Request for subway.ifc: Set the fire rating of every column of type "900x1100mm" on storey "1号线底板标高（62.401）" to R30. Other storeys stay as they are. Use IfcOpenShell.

First a look at what the model holds.

```python
import ifcopenshell
import ifcopenshell.util.element

model = ifcopenshell.open("subway.ifc")
print(model.schema)
storey = next(s for s in model.by_type("IfcBuildingStorey") if s.Name == "1号线底板标高（62.401）")
columns = [e for e in ifcopenshell.util.element.get_decomposition(storey) if e.is_a("IfcColumn")]
seen = {}
for e in columns:
    element_type = ifcopenshell.util.element.get_type(e)
    key = (element_type.Name if element_type != e and element_type else None, ifcopenshell.util.element.get_pset(e, "Pset_ColumnCommon", "FireRating"))
    seen[key] = seen.get(key, 0) + 1
for (name, value), count in sorted(seen.items(), key=str):
    print(count, "x", name, "|", value)
```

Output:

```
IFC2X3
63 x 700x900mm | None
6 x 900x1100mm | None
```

```python
import ifcopenshell
import ifcopenshell.api.pset
import ifcopenshell.util.element

model = ifcopenshell.open("subway.ifc")

storey = next(s for s in model.by_type("IfcBuildingStorey") if s.Name == "1号线底板标高（62.401）")
columns = [e for e in ifcopenshell.util.element.get_decomposition(storey) if e.is_a("IfcColumn")]

count = 0
for e in columns:
    element_type = ifcopenshell.util.element.get_type(e)
    if element_type in (None, e) or element_type.Name != "900x1100mm":
        continue
    # add_pset returns the element's existing set when there is one.
    pset = ifcopenshell.api.pset.add_pset(model, product=e, name="Pset_ColumnCommon")
    ifcopenshell.api.pset.edit_pset(model, pset=pset, properties={"FireRating": "R30"})
    count += 1

print(count, "columns updated")

model.write("subway_rev.ifc")
```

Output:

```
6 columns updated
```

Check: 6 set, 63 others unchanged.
